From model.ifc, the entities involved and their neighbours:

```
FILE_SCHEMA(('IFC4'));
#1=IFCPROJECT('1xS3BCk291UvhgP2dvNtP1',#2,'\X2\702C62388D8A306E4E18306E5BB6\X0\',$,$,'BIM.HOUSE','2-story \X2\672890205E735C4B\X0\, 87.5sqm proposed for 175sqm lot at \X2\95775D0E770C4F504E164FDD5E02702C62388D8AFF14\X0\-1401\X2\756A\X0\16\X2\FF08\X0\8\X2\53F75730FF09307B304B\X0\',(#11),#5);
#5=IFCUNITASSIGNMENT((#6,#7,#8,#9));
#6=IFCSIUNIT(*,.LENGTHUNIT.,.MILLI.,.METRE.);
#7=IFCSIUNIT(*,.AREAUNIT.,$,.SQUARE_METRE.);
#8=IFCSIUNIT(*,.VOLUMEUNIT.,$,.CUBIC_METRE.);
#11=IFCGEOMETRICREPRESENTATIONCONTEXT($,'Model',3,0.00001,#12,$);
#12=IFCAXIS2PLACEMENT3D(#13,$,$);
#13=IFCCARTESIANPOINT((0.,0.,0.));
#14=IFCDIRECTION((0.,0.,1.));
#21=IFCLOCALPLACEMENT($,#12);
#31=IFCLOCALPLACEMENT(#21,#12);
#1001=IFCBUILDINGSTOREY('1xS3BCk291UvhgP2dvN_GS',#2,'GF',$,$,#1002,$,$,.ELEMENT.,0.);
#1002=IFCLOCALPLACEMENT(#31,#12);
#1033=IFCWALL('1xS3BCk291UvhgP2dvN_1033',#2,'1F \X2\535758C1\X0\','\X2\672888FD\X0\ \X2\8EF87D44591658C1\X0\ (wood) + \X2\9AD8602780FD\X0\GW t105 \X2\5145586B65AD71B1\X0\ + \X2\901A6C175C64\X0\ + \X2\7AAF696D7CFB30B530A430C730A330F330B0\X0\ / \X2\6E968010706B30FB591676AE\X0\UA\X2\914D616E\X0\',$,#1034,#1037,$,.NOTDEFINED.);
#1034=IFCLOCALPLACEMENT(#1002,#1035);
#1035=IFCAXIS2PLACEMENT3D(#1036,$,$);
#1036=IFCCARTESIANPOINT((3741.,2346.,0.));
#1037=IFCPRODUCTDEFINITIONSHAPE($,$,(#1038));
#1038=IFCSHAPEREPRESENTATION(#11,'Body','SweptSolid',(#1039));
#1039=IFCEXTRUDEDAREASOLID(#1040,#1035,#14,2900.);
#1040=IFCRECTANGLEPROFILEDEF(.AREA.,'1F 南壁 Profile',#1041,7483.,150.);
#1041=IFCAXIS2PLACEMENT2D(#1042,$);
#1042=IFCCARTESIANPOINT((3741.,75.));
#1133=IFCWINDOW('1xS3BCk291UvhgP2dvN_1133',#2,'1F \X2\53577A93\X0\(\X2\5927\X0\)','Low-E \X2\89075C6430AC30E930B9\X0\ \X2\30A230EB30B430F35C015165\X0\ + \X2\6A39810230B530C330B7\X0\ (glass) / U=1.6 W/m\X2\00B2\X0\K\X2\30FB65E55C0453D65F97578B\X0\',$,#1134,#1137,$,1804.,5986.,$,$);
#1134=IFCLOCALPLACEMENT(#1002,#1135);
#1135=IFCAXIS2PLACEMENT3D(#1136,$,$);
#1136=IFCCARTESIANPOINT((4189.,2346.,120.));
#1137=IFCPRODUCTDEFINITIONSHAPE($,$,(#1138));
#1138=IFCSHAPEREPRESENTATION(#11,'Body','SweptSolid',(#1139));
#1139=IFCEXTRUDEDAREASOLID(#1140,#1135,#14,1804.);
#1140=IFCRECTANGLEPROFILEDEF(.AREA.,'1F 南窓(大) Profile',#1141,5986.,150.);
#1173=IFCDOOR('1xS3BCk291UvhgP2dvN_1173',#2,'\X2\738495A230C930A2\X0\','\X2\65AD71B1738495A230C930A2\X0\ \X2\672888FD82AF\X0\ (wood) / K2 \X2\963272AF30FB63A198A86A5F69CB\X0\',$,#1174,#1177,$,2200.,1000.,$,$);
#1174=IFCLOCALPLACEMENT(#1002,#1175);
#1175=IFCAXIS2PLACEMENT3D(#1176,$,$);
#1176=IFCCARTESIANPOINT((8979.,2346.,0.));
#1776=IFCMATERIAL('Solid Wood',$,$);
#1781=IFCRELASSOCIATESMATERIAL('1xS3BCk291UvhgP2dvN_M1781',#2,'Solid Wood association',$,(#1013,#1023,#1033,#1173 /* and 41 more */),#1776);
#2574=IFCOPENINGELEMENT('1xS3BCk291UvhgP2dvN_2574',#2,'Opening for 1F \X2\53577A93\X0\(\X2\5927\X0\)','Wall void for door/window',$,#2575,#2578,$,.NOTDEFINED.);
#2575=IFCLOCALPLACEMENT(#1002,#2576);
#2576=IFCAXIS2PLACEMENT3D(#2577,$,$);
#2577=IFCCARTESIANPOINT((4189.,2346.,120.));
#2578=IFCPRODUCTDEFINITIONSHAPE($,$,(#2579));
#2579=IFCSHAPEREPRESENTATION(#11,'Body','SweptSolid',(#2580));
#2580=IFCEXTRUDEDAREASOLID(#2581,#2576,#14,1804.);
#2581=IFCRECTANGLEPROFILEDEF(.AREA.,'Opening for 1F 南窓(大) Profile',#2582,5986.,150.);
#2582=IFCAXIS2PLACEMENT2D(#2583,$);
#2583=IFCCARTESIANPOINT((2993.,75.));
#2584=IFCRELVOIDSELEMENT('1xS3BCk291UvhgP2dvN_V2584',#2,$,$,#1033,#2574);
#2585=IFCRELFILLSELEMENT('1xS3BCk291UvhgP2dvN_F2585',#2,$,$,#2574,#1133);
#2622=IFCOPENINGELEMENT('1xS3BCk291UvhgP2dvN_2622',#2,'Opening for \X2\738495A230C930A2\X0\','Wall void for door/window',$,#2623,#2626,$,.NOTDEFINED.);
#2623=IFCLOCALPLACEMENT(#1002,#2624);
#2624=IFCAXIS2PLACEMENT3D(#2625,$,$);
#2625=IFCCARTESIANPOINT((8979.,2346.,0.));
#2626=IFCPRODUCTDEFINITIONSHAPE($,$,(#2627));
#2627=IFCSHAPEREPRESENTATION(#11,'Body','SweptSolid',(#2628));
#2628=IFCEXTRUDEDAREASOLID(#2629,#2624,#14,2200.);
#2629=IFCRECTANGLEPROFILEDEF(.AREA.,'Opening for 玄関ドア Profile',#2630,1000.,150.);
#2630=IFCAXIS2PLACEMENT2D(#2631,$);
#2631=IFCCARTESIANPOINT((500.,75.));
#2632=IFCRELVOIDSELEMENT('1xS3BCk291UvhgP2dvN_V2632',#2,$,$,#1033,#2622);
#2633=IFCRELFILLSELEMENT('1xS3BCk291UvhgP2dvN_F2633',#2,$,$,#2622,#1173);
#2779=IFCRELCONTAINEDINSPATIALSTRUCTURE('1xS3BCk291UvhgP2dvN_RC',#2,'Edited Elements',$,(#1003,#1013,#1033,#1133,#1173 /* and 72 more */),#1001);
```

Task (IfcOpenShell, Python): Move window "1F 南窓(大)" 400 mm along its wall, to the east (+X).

```python
import ifcopenshell
import ifcopenshell.api.geometry
import ifcopenshell.util.placement
import ifcopenshell.util.unit

model = ifcopenshell.open("model.ifc")
unit_scale = ifcopenshell.util.unit.calculate_unit_scale(model)

window = model.by_guid("1xS3BCk291UvhgP2dvN_1133")
opening = window.FillsVoids[0].RelatingOpeningElement
wall = opening.VoidsElements[0].RelatingBuildingElement

wall_matrix = ifcopenshell.util.placement.get_local_placement(wall.ObjectPlacement)
shift = wall_matrix[:3, 0] * 0.4 / unit_scale
before = ifcopenshell.util.placement.get_local_placement(window.ObjectPlacement)[:3, 3].copy()

# The window is not placed relative to its opening, so move both.
for product in (opening, window):
    matrix = ifcopenshell.util.placement.get_local_placement(product.ObjectPlacement)
    matrix[:3, 3] += shift
    ifcopenshell.api.geometry.edit_object_placement(model, product=product, matrix=matrix, is_si=False)

after = ifcopenshell.util.placement.get_local_placement(window.ObjectPlacement)[:3, 3]
print("window moved by", (after - before).round(3) + 0.0)

model.write("model_v2.ifc")
```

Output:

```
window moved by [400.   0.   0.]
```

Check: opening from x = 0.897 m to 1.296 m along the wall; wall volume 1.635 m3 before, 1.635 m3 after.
